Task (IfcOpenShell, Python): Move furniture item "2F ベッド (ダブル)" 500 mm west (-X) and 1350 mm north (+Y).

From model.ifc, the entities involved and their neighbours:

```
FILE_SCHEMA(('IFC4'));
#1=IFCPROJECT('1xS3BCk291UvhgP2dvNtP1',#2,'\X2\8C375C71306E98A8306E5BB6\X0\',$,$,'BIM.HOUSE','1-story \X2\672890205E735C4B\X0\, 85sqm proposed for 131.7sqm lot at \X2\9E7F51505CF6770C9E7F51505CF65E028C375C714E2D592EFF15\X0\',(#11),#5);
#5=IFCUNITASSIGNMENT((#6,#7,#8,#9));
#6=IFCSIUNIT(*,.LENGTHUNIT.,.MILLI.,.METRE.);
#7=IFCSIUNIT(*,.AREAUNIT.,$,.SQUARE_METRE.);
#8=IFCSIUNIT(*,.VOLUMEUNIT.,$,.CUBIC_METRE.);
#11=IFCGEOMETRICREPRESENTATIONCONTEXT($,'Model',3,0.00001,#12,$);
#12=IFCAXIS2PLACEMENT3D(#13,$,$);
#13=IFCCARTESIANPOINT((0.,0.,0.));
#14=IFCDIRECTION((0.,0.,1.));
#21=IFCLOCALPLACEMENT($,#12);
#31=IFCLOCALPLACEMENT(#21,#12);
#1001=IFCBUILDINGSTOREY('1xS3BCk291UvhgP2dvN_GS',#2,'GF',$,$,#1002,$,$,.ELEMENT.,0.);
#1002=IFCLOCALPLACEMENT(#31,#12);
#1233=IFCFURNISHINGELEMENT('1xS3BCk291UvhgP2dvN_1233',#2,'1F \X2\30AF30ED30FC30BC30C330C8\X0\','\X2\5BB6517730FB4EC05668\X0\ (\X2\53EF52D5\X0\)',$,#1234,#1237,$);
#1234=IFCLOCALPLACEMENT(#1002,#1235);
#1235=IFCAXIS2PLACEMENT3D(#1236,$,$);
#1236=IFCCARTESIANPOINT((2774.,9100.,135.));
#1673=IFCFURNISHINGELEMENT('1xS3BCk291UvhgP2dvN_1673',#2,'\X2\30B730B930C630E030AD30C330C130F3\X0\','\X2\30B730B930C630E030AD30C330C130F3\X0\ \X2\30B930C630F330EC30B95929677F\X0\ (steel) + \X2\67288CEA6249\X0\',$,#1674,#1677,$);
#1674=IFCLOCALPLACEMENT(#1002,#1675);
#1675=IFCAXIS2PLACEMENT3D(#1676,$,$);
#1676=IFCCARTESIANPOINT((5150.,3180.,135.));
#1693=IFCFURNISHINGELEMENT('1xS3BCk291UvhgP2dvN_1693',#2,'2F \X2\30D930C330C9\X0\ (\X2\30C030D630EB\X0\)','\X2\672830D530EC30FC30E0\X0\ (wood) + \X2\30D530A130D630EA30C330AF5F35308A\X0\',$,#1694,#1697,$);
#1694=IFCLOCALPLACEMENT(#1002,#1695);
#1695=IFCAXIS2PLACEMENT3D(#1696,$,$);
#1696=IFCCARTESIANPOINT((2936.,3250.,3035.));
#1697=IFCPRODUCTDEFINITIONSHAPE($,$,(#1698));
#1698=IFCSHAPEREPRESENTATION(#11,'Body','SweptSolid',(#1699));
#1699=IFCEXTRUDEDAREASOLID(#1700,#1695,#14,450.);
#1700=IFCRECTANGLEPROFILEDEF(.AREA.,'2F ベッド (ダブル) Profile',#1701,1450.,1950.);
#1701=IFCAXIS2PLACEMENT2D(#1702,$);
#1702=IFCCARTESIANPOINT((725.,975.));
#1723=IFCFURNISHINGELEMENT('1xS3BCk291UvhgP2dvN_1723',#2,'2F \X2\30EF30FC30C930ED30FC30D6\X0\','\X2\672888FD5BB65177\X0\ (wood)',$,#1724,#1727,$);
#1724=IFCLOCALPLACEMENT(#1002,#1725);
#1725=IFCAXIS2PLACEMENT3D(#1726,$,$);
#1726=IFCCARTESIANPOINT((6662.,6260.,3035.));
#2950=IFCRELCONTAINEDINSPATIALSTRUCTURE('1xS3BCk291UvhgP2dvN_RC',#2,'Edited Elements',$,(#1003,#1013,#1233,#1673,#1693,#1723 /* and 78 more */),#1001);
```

```python
import ifcopenshell
import ifcopenshell.api.geometry
import ifcopenshell.util.placement
import ifcopenshell.util.unit

model = ifcopenshell.open("model.ifc")
unit_scale = ifcopenshell.util.unit.calculate_unit_scale(model)

item = model.by_guid("1xS3BCk291UvhgP2dvN_1693")
matrix = ifcopenshell.util.placement.get_local_placement(item.ObjectPlacement)
matrix[0, 3] -= 0.5 / unit_scale
matrix[1, 3] += 1.35 / unit_scale
ifcopenshell.api.geometry.edit_object_placement(model, product=item, matrix=matrix, is_si=False)

print(ifcopenshell.util.placement.get_local_placement(item.ObjectPlacement).round(3) + 0.0)

model.write("model_v2.ifc")
```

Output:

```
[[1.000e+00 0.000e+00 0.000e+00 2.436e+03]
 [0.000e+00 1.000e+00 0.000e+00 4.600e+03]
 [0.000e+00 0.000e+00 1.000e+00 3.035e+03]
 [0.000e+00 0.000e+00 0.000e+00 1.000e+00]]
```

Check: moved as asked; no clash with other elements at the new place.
